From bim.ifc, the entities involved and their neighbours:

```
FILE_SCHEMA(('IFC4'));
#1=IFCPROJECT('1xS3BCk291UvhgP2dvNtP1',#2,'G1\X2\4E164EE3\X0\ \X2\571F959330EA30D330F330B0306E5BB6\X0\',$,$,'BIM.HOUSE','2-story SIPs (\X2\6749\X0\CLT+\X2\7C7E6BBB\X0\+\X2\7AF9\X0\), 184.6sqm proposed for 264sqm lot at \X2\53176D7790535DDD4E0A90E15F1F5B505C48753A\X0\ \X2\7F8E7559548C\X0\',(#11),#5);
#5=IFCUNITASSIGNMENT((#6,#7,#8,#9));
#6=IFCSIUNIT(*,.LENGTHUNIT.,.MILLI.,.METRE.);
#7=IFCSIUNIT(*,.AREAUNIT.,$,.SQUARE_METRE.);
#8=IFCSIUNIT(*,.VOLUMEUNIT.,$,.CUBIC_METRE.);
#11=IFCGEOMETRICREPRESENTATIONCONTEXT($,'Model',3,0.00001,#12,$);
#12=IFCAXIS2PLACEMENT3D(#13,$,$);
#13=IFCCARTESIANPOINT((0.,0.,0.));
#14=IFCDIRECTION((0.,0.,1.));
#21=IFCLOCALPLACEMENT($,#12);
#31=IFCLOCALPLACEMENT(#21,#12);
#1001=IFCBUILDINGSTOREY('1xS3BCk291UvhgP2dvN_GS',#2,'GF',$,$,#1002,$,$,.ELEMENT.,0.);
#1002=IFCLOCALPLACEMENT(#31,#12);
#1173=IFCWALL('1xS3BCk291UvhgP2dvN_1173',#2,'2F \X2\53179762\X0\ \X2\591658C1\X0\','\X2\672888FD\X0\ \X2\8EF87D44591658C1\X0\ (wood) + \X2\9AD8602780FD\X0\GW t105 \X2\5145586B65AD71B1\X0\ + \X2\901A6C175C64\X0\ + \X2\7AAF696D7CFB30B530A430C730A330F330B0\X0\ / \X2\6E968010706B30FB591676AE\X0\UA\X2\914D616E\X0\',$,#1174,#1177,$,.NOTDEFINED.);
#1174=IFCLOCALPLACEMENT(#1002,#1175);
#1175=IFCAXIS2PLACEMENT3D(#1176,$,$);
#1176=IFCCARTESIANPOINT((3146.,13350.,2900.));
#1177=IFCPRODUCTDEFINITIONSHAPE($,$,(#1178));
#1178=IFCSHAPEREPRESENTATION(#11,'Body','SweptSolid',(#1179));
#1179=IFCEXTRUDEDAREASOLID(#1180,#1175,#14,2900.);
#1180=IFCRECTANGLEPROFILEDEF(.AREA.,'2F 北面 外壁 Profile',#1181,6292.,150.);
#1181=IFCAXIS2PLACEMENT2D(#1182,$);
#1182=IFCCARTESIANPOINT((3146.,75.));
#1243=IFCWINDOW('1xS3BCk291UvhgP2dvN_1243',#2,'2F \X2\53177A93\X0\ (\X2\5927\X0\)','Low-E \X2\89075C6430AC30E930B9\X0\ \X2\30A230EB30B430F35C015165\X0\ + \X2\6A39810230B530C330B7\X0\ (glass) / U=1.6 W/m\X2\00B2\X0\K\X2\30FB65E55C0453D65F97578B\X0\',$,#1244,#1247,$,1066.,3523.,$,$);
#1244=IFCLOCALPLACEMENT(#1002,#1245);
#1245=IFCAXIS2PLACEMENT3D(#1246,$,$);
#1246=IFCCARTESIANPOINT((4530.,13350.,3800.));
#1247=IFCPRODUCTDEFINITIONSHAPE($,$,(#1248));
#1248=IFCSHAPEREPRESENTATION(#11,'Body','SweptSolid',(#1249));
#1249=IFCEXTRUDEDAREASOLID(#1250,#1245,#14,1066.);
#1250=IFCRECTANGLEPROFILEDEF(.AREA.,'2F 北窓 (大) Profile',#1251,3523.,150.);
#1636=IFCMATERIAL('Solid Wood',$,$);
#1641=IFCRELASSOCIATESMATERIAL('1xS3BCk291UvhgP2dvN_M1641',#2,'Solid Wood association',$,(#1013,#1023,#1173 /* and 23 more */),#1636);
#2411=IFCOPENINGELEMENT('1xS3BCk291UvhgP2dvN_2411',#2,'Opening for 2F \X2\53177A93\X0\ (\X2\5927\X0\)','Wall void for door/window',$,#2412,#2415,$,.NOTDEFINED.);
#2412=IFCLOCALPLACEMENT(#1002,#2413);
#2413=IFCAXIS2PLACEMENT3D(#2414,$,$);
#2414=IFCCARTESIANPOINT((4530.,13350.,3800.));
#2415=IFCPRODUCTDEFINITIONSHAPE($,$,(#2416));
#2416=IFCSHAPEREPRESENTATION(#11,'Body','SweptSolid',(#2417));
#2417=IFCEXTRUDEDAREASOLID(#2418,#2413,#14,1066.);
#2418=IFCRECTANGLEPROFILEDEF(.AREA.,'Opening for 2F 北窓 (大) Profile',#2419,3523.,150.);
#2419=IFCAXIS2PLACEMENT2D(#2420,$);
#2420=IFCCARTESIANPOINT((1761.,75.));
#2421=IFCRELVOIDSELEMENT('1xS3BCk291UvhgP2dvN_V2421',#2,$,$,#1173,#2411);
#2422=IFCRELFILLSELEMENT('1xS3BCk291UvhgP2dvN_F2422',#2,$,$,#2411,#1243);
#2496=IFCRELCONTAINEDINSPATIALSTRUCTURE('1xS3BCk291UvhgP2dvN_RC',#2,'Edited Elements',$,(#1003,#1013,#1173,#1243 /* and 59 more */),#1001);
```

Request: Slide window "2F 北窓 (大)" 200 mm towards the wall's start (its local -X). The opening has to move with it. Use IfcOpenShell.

```python
import ifcopenshell
import ifcopenshell.api.geometry
import ifcopenshell.util.placement
import ifcopenshell.util.unit

model = ifcopenshell.open("bim.ifc")
unit_scale = ifcopenshell.util.unit.calculate_unit_scale(model)

window = model.by_guid("1xS3BCk291UvhgP2dvN_1243")
opening = window.FillsVoids[0].RelatingOpeningElement
wall = opening.VoidsElements[0].RelatingBuildingElement

wall_matrix = ifcopenshell.util.placement.get_local_placement(wall.ObjectPlacement)
shift = wall_matrix[:3, 0] * -0.2 / unit_scale
before = ifcopenshell.util.placement.get_local_placement(window.ObjectPlacement)[:3, 3].copy()

# The window is not placed relative to its opening, so move both.
for product in (opening, window):
    matrix = ifcopenshell.util.placement.get_local_placement(product.ObjectPlacement)
    matrix[:3, 3] += shift
    ifcopenshell.api.geometry.edit_object_placement(model, product=product, matrix=matrix, is_si=False)

after = ifcopenshell.util.placement.get_local_placement(window.ObjectPlacement)[:3, 3]
print("window moved by", (after - before).round(3) + 0.0)

model.write("bim_rev.ifc")
```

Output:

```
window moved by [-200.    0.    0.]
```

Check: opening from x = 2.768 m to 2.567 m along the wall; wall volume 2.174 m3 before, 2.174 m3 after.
